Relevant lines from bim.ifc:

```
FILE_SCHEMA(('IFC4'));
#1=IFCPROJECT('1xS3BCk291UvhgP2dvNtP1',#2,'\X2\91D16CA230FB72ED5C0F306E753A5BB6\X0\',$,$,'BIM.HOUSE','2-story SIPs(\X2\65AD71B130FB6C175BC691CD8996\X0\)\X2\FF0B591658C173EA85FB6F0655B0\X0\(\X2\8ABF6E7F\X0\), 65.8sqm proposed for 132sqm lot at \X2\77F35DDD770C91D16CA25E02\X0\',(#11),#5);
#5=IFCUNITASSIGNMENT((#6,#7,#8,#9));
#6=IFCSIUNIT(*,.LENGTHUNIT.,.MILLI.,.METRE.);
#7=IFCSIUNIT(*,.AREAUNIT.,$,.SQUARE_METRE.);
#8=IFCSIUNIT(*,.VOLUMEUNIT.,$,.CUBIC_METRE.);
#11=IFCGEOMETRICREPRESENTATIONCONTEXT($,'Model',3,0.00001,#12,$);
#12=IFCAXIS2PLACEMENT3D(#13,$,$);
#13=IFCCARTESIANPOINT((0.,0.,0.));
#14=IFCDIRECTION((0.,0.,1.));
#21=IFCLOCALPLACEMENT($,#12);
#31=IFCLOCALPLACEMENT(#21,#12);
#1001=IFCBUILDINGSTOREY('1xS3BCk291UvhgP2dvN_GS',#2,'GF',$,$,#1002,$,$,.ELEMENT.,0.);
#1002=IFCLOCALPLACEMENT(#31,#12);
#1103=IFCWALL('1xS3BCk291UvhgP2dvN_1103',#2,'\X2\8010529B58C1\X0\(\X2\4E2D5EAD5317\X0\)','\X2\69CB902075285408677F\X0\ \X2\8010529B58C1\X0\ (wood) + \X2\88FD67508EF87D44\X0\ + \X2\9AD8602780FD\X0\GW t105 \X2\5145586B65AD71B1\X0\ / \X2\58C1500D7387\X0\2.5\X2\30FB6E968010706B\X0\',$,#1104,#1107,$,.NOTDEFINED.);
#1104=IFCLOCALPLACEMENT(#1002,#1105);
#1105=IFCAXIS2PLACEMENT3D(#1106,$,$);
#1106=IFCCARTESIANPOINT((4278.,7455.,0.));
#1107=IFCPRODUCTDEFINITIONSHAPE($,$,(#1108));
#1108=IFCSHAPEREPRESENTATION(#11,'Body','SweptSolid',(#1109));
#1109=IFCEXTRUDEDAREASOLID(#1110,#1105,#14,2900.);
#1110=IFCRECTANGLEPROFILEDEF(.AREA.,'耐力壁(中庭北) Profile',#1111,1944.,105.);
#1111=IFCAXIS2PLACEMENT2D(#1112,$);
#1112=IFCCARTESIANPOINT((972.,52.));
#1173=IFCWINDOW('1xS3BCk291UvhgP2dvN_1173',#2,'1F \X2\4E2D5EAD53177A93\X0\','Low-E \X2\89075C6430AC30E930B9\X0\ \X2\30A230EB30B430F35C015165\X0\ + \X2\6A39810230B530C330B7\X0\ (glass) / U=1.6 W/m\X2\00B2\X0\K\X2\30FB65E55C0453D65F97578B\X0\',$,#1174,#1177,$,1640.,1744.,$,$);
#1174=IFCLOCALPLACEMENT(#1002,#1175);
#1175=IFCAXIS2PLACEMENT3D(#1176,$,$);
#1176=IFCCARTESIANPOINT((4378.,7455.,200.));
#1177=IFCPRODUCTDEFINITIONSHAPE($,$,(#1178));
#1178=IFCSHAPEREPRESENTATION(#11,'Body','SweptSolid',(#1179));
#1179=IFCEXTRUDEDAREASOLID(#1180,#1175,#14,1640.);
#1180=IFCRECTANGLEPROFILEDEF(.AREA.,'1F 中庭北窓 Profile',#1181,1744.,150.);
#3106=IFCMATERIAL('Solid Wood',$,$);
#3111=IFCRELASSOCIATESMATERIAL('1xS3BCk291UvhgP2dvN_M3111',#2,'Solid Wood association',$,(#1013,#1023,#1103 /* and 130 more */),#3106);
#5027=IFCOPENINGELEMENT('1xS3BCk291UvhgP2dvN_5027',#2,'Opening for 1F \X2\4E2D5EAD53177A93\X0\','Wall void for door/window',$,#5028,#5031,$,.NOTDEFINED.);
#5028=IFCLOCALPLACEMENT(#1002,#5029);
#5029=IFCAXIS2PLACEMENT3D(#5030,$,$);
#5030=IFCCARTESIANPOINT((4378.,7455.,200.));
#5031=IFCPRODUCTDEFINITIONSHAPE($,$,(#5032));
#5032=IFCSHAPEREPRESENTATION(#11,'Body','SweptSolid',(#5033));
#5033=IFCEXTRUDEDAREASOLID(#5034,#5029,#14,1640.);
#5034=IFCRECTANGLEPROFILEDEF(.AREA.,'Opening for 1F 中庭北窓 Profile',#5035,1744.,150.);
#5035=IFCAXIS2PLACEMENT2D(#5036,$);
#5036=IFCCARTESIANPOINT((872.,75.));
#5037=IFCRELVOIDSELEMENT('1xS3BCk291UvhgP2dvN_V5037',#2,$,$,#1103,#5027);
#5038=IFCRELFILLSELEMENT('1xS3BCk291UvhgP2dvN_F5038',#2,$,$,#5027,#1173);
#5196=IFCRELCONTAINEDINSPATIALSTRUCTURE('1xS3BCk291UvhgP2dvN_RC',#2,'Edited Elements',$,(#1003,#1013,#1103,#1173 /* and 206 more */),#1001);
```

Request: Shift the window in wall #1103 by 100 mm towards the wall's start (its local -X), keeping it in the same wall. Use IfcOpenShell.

```python
import ifcopenshell
import ifcopenshell.api.geometry
import ifcopenshell.util.placement
import ifcopenshell.util.unit

model = ifcopenshell.open("bim.ifc")
unit_scale = ifcopenshell.util.unit.calculate_unit_scale(model)

window = model.by_guid("1xS3BCk291UvhgP2dvN_1173")
opening = window.FillsVoids[0].RelatingOpeningElement
wall = opening.VoidsElements[0].RelatingBuildingElement

wall_matrix = ifcopenshell.util.placement.get_local_placement(wall.ObjectPlacement)
shift = wall_matrix[:3, 0] * -0.1 / unit_scale
before = ifcopenshell.util.placement.get_local_placement(window.ObjectPlacement)[:3, 3].copy()

# The window is not placed relative to its opening, so move both.
for product in (opening, window):
    matrix = ifcopenshell.util.placement.get_local_placement(product.ObjectPlacement)
    matrix[:3, 3] += shift
    ifcopenshell.api.geometry.edit_object_placement(model, product=product, matrix=matrix, is_si=False)

after = ifcopenshell.util.placement.get_local_placement(window.ObjectPlacement)[:3, 3]
print("window moved by", (after - before).round(3) + 0.0)

model.write("bim_v2.ifc")
```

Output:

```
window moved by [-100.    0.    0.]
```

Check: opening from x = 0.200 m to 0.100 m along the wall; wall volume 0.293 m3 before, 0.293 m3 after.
